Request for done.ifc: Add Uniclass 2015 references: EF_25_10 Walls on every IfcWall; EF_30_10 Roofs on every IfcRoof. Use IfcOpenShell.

First a look at what the model holds.

```python
import ifcopenshell

model = ifcopenshell.open("done.ifc")
print(model.schema)
print("classifications:", [c.Name for c in model.by_type("IfcClassification")])
for ifc_class in ("IfcDoor", "IfcRoof", "IfcStair", "IfcWall", "IfcWindow"):
    print(ifc_class, len(model.by_type(ifc_class)))
```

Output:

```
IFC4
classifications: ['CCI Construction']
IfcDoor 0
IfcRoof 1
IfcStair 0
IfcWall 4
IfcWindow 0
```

```python
import ifcopenshell
import ifcopenshell.api.classification

model = ifcopenshell.open("done.ifc")

system = ifcopenshell.api.classification.add_classification(model, classification="Uniclass 2015")

codes = {
    "IfcWall": ("EF_25_10", "Walls"),
    "IfcRoof": ("EF_30_10", "Roofs"),
}
for ifc_class, (code, name) in codes.items():
    products = model.by_type(ifc_class)
    ifcopenshell.api.classification.add_reference(
        model, products=products, classification=system, identification=code, name=name
    )
    print(code, len(products))

model.write("done_rev.ifc")
```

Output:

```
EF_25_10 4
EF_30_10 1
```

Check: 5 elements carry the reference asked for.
